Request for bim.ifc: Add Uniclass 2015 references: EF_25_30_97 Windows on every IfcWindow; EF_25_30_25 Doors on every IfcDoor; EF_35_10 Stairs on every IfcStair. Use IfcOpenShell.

First a look at what the model holds.

```python
import ifcopenshell

model = ifcopenshell.open("bim.ifc")
print(model.schema)
print("classifications:", [c.Name for c in model.by_type("IfcClassification")])
for ifc_class in ("IfcDoor", "IfcRoof", "IfcStair", "IfcWall", "IfcWindow"):
    print(ifc_class, len(model.by_type(ifc_class)))
```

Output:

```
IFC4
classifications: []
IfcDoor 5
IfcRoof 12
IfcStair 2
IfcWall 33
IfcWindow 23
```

```python
import ifcopenshell
import ifcopenshell.api.classification

model = ifcopenshell.open("bim.ifc")

system = ifcopenshell.api.classification.add_classification(model, classification="Uniclass 2015")

codes = {
    "IfcWindow": ("EF_25_30_97", "Windows"),
    "IfcDoor": ("EF_25_30_25", "Doors"),
    "IfcStair": ("EF_35_10", "Stairs"),
}
for ifc_class, (code, name) in codes.items():
    products = model.by_type(ifc_class)
    ifcopenshell.api.classification.add_reference(
        model, products=products, classification=system, identification=code, name=name
    )
    print(code, len(products))

model.write("bim-out.ifc")
```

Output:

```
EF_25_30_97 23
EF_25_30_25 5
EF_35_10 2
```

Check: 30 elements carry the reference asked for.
